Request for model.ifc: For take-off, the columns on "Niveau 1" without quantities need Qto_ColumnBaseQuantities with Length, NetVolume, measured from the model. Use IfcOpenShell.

First a look at what the model holds.

```python
import ifcopenshell
import ifcopenshell.util.element
import ifcopenshell.util.unit

model = ifcopenshell.open("model.ifc")
print(model.schema)
for unit_type in ("LENGTHUNIT", "AREAUNIT", "VOLUMEUNIT"):
    print(unit_type, ifcopenshell.util.unit.calculate_unit_scale(model, unit_type))
storey = next(s for s in model.by_type("IfcBuildingStorey") if s.Name == "Niveau 1")
columns = [e for e in ifcopenshell.util.element.get_decomposition(storey) if e.is_a("IfcColumn")]
for e in sorted(columns, key=lambda e: e.id()):
    print(e.id(), e.is_a(), e.Name, list(ifcopenshell.util.element.get_psets(e, qtos_only=True)), sep=" | ")
```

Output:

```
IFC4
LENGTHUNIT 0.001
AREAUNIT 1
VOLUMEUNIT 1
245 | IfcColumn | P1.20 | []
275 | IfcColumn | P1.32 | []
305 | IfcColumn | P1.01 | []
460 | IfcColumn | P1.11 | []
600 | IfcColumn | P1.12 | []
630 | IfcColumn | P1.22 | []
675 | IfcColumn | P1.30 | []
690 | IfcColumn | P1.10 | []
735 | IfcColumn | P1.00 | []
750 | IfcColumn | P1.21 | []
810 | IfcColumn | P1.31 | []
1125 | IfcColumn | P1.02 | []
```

```python
import ifcopenshell
import ifcopenshell.api.pset
import ifcopenshell.geom
import ifcopenshell.util.element
import ifcopenshell.util.shape
import ifcopenshell.util.unit

model = ifcopenshell.open("model.ifc")
unit_scale = ifcopenshell.util.unit.calculate_unit_scale(model)
volume_scale = ifcopenshell.util.unit.calculate_unit_scale(model, "VOLUMEUNIT")
settings = ifcopenshell.geom.settings()

storey = next(s for s in model.by_type("IfcBuildingStorey") if s.Name == "Niveau 1")
columns = [e for e in ifcopenshell.util.element.get_decomposition(storey) if e.is_a("IfcColumn")]

for e in sorted(columns, key=lambda e: e.id()):
    if ifcopenshell.util.element.get_psets(e, qtos_only=True, should_inherit=False):
        continue
    # Geometry comes back in metres, in the element's own axes.
    shape = ifcopenshell.geom.create_shape(settings, e)
    values = {
        "Length": ifcopenshell.util.shape.get_z(shape.geometry) / unit_scale,
        "NetVolume": ifcopenshell.util.shape.get_volume(shape.geometry) / volume_scale,
    }
    qto = ifcopenshell.api.pset.add_qto(model, product=e, name="Qto_ColumnBaseQuantities")
    ifcopenshell.api.pset.edit_qto(model, qto=qto, properties=values)
    print(e.id(), {k: round(v, 3) for k, v in values.items()})

model.write("model_rev.ifc")
```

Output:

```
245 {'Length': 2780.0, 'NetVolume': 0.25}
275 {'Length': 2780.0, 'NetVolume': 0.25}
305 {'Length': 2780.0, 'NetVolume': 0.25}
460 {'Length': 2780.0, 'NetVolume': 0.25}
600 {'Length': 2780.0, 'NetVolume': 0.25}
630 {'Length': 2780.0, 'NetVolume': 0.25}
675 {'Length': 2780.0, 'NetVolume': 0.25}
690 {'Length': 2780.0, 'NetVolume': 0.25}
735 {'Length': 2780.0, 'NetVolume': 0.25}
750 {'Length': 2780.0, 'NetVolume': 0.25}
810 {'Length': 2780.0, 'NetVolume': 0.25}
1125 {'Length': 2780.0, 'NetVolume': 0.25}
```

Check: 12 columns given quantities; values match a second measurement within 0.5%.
